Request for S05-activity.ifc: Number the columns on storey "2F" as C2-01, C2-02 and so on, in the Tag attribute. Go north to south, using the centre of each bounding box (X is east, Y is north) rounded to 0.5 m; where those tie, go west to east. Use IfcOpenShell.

First a look at what the model holds.

```python
import ifcopenshell
import ifcopenshell.util.element
import ifcopenshell.util.placement

model = ifcopenshell.open("S05-activity.ifc")
print(model.schema)
storey = next(s for s in model.by_type("IfcBuildingStorey") if s.Name == "2F")
columns = [e for e in ifcopenshell.util.element.get_decomposition(storey) if e.is_a("IfcColumn")]
for e in sorted(columns, key=lambda e: e.id()):
    origin = ifcopenshell.util.placement.get_local_placement(e.ObjectPlacement)[:3, 3]
    print(e.id(), e.Tag, e.Name, origin.round(2) + 0.0, sep=" | ")
```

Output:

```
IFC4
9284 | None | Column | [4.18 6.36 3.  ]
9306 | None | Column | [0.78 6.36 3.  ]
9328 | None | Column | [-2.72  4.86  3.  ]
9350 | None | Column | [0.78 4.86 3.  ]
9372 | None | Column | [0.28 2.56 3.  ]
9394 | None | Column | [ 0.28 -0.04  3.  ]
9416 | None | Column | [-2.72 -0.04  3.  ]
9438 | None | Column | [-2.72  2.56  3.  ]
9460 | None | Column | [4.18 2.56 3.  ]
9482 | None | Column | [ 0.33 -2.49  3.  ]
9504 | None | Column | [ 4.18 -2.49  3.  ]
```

```python
import ifcopenshell
import ifcopenshell.geom
import ifcopenshell.util.element
import ifcopenshell.util.shape

model = ifcopenshell.open("S05-activity.ifc")
settings = ifcopenshell.geom.settings()
settings.set("use-world-coords", True)


def centre(element):
    shape = ifcopenshell.geom.create_shape(settings, element)
    return ifcopenshell.util.shape.get_bbox_centroid(shape.geometry)


storey = next(s for s in model.by_type("IfcBuildingStorey") if s.Name == "2F")
columns = [e for e in ifcopenshell.util.element.get_decomposition(storey) if e.is_a("IfcColumn")]

# Insertion points can sit at a corner or the storey origin, so sort by the geometry (in metres).
centres = {e: centre(e) for e in columns}
columns.sort(key=lambda e: (-round(centres[e][1] / 0.5), centres[e][0]))

for i, e in enumerate(columns, start=1):
    number = f"C2-{i:02d}"
    e.Tag = number
    print(e.id(), number)

model.write("S05-activity_rev.ifc")
```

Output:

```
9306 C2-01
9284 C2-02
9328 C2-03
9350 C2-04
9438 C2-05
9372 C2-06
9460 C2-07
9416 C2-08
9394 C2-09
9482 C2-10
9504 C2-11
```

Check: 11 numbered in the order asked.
